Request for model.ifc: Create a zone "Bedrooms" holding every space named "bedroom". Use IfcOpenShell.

First a look at what the model holds.

```python
import ifcopenshell

model = ifcopenshell.open("model.ifc")
print(model.schema)
seen = {}
for space in model.by_type("IfcSpace"):
    seen[space.LongName] = seen.get(space.LongName, 0) + 1
for name, count in sorted(seen.items(), key=str):
    print(count, "x", name)
print("zones:", [z.Name for z in model.by_type("IfcZone")][:20])
```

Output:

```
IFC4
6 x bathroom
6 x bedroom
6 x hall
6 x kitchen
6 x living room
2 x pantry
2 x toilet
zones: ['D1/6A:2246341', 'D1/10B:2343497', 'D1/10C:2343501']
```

```python
import ifcopenshell
import ifcopenshell.api.group
import ifcopenshell.api.root

model = ifcopenshell.open("model.ifc")

names = {"bedroom"}
spaces = [s for s in model.by_type("IfcSpace") if s.LongName in names]

zone = ifcopenshell.api.root.create_entity(model, ifc_class="IfcZone", name="Bedrooms")
ifcopenshell.api.group.assign_group(model, products=spaces, group=zone)
print(len(spaces), "spaces in", zone.Name)

model.write("model-out.ifc")
```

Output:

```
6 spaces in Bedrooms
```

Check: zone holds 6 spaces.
